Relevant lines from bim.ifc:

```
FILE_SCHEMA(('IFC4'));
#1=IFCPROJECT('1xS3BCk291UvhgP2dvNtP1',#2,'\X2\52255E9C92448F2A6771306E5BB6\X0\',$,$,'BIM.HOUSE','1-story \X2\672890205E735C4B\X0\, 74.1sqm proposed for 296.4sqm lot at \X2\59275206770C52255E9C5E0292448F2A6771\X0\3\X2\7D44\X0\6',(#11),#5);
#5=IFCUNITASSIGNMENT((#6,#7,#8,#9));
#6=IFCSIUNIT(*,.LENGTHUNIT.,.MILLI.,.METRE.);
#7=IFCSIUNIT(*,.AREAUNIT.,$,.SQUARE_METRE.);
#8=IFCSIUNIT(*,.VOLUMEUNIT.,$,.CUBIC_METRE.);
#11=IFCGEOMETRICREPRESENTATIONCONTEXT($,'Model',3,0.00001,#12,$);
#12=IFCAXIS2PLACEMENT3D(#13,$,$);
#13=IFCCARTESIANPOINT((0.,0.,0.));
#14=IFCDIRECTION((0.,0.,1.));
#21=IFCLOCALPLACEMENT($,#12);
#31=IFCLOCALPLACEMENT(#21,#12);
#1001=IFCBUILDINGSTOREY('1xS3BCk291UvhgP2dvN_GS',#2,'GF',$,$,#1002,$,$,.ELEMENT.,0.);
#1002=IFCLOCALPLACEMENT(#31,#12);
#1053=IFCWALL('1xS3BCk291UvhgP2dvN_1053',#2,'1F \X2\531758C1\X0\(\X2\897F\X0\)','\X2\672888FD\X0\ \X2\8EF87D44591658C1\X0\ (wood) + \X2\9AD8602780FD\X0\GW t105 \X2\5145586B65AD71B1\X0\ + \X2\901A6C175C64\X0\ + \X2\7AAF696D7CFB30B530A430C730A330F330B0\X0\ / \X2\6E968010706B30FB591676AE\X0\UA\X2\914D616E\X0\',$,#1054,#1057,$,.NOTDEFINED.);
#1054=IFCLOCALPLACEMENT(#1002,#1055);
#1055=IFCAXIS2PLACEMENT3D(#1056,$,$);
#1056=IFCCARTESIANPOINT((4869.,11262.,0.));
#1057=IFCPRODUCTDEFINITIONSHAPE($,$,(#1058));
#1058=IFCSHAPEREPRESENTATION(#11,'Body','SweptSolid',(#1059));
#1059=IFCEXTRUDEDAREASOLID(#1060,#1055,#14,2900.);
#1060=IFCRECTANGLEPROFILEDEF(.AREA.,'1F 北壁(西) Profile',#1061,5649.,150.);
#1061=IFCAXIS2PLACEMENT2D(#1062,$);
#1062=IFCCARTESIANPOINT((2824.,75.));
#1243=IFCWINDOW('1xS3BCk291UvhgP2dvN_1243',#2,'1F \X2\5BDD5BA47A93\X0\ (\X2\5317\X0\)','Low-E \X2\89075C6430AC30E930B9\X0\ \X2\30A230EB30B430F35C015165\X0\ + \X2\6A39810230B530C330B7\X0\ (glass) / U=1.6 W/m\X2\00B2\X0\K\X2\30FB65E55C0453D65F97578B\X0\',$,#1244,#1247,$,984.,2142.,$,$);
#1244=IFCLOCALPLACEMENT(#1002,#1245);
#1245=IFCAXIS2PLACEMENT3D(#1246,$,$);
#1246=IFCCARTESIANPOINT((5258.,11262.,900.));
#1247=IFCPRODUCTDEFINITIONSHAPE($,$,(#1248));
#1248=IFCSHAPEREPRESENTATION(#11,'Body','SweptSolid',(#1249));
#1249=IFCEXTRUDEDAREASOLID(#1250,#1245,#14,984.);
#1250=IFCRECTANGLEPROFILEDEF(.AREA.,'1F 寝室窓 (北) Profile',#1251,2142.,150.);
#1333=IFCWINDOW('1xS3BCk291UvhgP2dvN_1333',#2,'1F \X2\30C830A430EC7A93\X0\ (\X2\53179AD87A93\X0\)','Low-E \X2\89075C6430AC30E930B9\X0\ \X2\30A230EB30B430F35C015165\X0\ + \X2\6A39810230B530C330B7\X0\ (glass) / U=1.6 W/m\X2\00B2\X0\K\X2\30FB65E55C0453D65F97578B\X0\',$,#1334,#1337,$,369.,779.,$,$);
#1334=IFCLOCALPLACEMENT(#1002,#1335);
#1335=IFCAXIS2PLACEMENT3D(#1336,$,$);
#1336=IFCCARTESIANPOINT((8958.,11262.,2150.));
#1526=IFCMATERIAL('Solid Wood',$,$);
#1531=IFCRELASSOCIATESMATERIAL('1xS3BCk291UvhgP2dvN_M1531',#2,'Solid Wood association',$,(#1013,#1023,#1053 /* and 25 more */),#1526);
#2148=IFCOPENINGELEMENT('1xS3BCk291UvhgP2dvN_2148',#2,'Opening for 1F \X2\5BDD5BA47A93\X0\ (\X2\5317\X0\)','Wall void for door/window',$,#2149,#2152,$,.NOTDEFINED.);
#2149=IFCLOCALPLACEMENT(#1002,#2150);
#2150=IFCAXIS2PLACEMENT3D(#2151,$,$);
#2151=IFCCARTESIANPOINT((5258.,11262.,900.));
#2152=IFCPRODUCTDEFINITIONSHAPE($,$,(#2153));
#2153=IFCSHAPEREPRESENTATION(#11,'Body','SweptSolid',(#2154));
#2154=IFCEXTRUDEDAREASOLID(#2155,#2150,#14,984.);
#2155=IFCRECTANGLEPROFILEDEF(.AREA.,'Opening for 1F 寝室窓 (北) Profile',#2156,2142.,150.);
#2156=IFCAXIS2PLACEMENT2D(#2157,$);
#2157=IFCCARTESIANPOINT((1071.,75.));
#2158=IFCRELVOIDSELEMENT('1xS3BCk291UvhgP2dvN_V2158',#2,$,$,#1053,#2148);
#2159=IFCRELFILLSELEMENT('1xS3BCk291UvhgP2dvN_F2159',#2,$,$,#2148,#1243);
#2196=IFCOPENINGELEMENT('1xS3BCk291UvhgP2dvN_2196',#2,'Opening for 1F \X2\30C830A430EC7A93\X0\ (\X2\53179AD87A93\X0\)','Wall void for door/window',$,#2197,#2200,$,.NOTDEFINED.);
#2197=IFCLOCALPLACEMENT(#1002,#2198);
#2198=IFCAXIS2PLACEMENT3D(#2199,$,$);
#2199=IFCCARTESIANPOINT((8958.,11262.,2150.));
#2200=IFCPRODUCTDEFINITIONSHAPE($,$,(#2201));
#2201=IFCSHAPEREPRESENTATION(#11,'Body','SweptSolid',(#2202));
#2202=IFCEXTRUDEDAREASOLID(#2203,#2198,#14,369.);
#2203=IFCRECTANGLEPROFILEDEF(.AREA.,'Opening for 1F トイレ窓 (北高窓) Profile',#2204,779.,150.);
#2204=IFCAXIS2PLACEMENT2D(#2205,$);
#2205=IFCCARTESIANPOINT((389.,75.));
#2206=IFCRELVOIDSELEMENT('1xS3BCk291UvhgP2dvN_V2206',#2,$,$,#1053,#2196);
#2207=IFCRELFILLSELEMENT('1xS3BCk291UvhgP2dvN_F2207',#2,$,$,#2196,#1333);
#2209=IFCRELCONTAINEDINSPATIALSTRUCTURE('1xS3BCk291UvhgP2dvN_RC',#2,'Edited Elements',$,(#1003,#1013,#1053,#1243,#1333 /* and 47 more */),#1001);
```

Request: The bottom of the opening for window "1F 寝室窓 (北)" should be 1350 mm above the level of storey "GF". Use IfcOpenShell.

```python
import numpy as np
import ifcopenshell
import ifcopenshell.api.geometry
import ifcopenshell.geom
import ifcopenshell.util.element
import ifcopenshell.util.placement
import ifcopenshell.util.shape
import ifcopenshell.util.unit

model = ifcopenshell.open("bim.ifc")
unit_scale = ifcopenshell.util.unit.calculate_unit_scale(model)

window = model.by_id(1243)
opening = window.FillsVoids[0].RelatingOpeningElement
storey = ifcopenshell.util.element.get_container(window, ifc_class="IfcBuildingStorey")
level = ifcopenshell.util.placement.get_local_placement(storey.ObjectPlacement)[2, 3]

# The opening's origin need not be at the sill, so measure its lowest point.
shape = ifcopenshell.geom.create_shape(ifcopenshell.geom.settings(), opening)
bottom = ifcopenshell.util.shape.get_shape_bottom_elevation(shape, shape.geometry) / unit_scale
dz = level + 1350.0 - bottom

shift = np.array([0.0, 0.0, dz])
# The window is not placed relative to its opening, so move both.
for product in (opening, window):
    matrix = ifcopenshell.util.placement.get_local_placement(product.ObjectPlacement)
    matrix[:3, 3] += shift
    ifcopenshell.api.geometry.edit_object_placement(model, product=product, matrix=matrix, is_si=False)

print(f"moved by {dz * unit_scale:+.3f} m")

model.write("bim_rev.ifc")
```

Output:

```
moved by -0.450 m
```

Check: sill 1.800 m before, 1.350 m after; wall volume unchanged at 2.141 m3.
